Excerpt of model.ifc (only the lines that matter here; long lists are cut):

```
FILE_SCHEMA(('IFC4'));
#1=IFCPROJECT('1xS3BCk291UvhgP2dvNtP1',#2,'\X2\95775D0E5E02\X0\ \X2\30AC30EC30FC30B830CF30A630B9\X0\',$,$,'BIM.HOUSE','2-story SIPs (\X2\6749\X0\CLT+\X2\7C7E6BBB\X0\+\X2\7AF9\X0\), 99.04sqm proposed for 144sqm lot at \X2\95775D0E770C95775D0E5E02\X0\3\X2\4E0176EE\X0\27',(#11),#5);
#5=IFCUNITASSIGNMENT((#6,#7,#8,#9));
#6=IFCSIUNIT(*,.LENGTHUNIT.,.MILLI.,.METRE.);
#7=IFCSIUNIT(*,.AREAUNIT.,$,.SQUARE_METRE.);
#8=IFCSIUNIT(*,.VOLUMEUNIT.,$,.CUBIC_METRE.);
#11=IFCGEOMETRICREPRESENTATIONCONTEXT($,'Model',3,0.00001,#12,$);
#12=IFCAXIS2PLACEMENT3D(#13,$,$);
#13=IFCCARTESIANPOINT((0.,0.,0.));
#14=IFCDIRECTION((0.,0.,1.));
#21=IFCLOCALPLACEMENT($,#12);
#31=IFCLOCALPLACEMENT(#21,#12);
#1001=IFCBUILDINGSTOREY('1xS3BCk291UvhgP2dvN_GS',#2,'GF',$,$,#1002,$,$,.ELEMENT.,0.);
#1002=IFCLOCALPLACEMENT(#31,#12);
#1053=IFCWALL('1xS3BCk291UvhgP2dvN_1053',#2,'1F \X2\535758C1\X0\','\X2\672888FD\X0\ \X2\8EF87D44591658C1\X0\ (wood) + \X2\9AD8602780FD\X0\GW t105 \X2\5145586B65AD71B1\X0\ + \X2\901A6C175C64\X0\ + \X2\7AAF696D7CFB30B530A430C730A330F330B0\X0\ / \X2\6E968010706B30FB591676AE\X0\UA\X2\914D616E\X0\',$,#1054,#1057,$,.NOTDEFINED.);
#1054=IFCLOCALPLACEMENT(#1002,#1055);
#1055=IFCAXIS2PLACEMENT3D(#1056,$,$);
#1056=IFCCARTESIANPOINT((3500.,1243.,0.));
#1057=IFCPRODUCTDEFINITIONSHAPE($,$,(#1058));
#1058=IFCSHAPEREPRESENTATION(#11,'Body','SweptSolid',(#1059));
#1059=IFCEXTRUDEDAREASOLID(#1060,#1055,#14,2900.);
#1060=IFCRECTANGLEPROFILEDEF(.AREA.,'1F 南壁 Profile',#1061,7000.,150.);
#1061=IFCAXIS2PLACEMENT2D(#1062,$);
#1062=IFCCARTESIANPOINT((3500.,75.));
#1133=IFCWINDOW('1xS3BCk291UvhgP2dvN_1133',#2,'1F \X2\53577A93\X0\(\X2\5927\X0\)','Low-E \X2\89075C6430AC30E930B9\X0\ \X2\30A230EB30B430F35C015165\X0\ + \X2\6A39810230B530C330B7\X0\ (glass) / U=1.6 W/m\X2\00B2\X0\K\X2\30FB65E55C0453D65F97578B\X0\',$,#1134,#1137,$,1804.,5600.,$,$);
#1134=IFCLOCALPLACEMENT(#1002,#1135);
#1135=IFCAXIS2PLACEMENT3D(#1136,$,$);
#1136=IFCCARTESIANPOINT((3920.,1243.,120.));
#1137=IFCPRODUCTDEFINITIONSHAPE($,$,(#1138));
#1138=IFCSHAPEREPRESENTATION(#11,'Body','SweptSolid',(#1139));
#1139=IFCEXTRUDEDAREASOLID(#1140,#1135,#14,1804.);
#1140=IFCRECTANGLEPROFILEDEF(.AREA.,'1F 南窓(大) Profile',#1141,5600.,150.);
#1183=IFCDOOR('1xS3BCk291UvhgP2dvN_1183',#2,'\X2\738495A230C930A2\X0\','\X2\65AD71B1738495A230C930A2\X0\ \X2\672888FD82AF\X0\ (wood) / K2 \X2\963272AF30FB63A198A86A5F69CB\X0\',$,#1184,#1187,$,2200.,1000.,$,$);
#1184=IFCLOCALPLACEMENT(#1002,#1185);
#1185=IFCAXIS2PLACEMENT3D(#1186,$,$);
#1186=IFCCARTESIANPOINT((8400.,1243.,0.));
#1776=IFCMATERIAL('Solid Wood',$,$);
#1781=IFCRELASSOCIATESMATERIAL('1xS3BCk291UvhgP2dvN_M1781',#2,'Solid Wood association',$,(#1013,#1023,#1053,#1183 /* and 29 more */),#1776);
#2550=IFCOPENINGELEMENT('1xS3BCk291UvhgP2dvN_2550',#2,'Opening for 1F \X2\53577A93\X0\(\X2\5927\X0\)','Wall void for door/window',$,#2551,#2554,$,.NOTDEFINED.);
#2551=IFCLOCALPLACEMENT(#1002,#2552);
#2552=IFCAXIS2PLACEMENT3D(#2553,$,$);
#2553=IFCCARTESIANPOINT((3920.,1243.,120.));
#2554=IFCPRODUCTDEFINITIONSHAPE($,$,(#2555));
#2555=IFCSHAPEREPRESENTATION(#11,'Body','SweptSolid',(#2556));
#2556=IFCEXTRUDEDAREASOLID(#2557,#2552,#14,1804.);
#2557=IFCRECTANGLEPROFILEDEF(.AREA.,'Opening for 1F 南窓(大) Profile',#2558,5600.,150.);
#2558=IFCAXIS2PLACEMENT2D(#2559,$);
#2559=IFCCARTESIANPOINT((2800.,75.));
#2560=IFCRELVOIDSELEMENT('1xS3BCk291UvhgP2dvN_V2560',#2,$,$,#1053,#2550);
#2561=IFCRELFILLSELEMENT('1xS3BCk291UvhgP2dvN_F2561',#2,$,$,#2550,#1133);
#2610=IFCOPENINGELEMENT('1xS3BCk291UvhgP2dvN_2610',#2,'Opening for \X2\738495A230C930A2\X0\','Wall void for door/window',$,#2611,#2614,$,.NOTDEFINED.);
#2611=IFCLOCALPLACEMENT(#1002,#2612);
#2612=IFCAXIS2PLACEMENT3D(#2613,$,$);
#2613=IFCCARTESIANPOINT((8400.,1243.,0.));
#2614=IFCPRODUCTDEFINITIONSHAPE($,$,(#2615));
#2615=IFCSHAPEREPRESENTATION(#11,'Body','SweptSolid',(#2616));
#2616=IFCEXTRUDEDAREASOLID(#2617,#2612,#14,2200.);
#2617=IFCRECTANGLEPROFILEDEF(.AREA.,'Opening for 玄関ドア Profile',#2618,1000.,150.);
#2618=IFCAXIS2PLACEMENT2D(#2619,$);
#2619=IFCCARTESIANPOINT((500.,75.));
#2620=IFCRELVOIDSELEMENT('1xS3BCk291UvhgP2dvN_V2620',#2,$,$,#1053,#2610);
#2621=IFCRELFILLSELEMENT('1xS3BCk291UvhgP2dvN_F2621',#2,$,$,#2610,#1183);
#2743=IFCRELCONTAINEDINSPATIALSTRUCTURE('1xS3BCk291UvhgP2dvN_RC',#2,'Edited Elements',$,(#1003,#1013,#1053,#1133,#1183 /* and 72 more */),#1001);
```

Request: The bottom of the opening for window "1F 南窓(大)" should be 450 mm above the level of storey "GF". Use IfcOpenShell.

```python
import numpy as np
import ifcopenshell
import ifcopenshell.api.geometry
import ifcopenshell.geom
import ifcopenshell.util.element
import ifcopenshell.util.placement
import ifcopenshell.util.shape
import ifcopenshell.util.unit

model = ifcopenshell.open("model.ifc")
unit_scale = ifcopenshell.util.unit.calculate_unit_scale(model)

window = model.by_guid("1xS3BCk291UvhgP2dvN_1133")
opening = window.FillsVoids[0].RelatingOpeningElement
storey = ifcopenshell.util.element.get_container(window, ifc_class="IfcBuildingStorey")
level = ifcopenshell.util.placement.get_local_placement(storey.ObjectPlacement)[2, 3]

# The opening's origin need not be at the sill, so measure its lowest point.
shape = ifcopenshell.geom.create_shape(ifcopenshell.geom.settings(), opening)
bottom = ifcopenshell.util.shape.get_shape_bottom_elevation(shape, shape.geometry) / unit_scale
dz = level + 450.0 - bottom

shift = np.array([0.0, 0.0, dz])
# The window is not placed relative to its opening, so move both.
for product in (opening, window):
    matrix = ifcopenshell.util.placement.get_local_placement(product.ObjectPlacement)
    matrix[:3, 3] += shift
    ifcopenshell.api.geometry.edit_object_placement(model, product=product, matrix=matrix, is_si=False)

print(f"moved by {dz * unit_scale:+.3f} m")

model.write("model_v2.ifc")
```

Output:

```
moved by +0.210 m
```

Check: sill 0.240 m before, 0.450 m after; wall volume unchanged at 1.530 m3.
